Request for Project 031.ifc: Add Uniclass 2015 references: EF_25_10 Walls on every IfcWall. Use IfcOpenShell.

First a look at what the model holds.

```python
import ifcopenshell

model = ifcopenshell.open("Project 031.ifc")
print(model.schema)
print("classifications:", [c.Name for c in model.by_type("IfcClassification")])
for ifc_class in ("IfcDoor", "IfcRoof", "IfcStair", "IfcWall", "IfcWindow"):
    print(ifc_class, len(model.by_type(ifc_class)))
```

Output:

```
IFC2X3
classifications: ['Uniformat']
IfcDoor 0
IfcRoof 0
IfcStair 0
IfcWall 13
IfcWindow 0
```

```python
import ifcopenshell
import ifcopenshell.api.classification

model = ifcopenshell.open("Project 031.ifc")

# IFC2X3 requires Source and Edition and has no link from the project to the system.
system = model.create_entity("IfcClassification", Source="NBS", Edition="2015", Name="Uniclass 2015")

codes = {
    "IfcWall": ("EF_25_10", "Walls"),
}
for ifc_class, (code, name) in codes.items():
    products = model.by_type(ifc_class)
    ifcopenshell.api.classification.add_reference(
        model, products=products, classification=system, identification=code, name=name
    )
    print(code, len(products))

model.write("Project 031_edited.ifc")
```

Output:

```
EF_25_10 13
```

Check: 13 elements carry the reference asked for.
